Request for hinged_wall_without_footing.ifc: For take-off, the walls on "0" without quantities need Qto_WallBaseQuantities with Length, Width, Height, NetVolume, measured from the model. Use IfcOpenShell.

First a look at what the model holds.

```python
import ifcopenshell
import ifcopenshell.util.element
import ifcopenshell.util.unit

model = ifcopenshell.open("hinged_wall_without_footing.ifc")
print(model.schema)
for unit_type in ("LENGTHUNIT", "AREAUNIT", "VOLUMEUNIT"):
    print(unit_type, ifcopenshell.util.unit.calculate_unit_scale(model, unit_type))
storey = next(s for s in model.by_type("IfcBuildingStorey") if s.Name == "0")
walls = [e for e in ifcopenshell.util.element.get_decomposition(storey) if e.is_a("IfcWall")]
for e in sorted(walls, key=lambda e: e.id()):
    print(e.id(), e.is_a(), e.Name, list(ifcopenshell.util.element.get_psets(e, qtos_only=True)), sep=" | ")
```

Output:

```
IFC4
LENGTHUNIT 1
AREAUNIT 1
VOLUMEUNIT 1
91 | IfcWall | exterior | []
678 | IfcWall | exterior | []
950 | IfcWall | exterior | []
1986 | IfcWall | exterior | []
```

```python
import ifcopenshell
import ifcopenshell.api.pset
import ifcopenshell.geom
import ifcopenshell.util.element
import ifcopenshell.util.shape
import ifcopenshell.util.unit

model = ifcopenshell.open("hinged_wall_without_footing.ifc")
unit_scale = ifcopenshell.util.unit.calculate_unit_scale(model)
volume_scale = ifcopenshell.util.unit.calculate_unit_scale(model, "VOLUMEUNIT")
settings = ifcopenshell.geom.settings()

storey = next(s for s in model.by_type("IfcBuildingStorey") if s.Name == "0")
walls = [e for e in ifcopenshell.util.element.get_decomposition(storey) if e.is_a("IfcWall")]

for e in sorted(walls, key=lambda e: e.id()):
    if ifcopenshell.util.element.get_psets(e, qtos_only=True, should_inherit=False):
        continue
    # Geometry comes back in metres, in the element's own axes.
    shape = ifcopenshell.geom.create_shape(settings, e)
    values = {
        "Length": ifcopenshell.util.shape.get_x(shape.geometry) / unit_scale,
        "Width": ifcopenshell.util.shape.get_y(shape.geometry) / unit_scale,
        "Height": ifcopenshell.util.shape.get_z(shape.geometry) / unit_scale,
        "NetVolume": ifcopenshell.util.shape.get_volume(shape.geometry) / volume_scale,
    }
    qto = ifcopenshell.api.pset.add_qto(model, product=e, name="Qto_WallBaseQuantities")
    ifcopenshell.api.pset.edit_qto(model, qto=qto, properties=values)
    print(e.id(), {k: round(v, 3) for k, v in values.items()})

model.write("hinged_wall_without_footing_updated.ifc")
```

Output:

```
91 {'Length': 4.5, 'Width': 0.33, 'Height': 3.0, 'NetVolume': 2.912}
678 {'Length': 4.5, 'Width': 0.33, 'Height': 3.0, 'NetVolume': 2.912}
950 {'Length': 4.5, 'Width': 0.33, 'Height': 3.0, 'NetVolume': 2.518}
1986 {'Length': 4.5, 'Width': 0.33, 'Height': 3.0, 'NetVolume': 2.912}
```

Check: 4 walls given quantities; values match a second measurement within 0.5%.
